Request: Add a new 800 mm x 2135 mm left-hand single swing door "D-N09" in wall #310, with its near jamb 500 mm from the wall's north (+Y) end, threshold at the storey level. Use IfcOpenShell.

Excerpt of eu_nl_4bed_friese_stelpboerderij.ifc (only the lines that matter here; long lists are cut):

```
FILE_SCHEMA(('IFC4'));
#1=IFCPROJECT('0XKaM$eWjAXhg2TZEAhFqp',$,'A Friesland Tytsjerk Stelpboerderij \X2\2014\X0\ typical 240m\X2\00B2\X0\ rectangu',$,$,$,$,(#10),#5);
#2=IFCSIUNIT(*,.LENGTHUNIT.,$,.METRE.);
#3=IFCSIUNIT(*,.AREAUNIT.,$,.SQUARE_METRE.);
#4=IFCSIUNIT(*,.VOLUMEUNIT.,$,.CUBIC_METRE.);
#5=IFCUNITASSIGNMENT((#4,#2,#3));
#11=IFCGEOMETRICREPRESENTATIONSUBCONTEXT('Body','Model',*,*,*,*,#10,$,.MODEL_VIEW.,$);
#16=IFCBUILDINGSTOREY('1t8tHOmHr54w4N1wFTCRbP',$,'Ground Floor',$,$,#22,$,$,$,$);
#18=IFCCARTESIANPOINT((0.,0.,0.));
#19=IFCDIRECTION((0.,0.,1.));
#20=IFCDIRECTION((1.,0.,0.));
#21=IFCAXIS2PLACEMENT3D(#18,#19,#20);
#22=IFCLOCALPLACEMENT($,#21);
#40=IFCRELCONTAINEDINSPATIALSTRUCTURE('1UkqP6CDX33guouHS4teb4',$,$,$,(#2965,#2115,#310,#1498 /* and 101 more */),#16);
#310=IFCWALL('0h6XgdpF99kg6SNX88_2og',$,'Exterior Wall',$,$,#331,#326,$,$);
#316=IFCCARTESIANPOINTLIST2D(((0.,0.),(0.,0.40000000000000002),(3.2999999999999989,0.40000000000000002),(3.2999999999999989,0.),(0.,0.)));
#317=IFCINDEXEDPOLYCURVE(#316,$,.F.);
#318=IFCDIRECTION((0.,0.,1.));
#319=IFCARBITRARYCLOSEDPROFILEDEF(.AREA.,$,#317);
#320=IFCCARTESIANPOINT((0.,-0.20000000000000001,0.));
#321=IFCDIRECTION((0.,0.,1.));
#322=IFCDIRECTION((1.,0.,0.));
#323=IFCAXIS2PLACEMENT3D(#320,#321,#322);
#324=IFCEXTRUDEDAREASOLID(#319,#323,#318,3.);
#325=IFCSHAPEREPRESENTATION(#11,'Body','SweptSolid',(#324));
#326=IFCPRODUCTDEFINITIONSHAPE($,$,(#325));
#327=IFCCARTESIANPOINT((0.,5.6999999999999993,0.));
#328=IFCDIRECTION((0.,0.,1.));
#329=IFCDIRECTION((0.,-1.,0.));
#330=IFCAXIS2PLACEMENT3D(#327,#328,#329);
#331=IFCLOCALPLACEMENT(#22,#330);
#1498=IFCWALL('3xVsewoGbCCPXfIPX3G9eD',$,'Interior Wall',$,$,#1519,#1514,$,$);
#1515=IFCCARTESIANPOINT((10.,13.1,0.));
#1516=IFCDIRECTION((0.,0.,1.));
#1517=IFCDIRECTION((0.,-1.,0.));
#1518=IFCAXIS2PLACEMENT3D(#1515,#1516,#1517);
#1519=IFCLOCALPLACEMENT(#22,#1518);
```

```python
import numpy as np
import ifcopenshell
import ifcopenshell.api.feature
import ifcopenshell.api.geometry
import ifcopenshell.api.root
import ifcopenshell.api.spatial
import ifcopenshell.geom
import ifcopenshell.util.element
import ifcopenshell.util.placement
import ifcopenshell.util.representation
import ifcopenshell.util.shape
import ifcopenshell.util.unit

model = ifcopenshell.open("eu_nl_4bed_friese_stelpboerderij.ifc")
unit_scale = ifcopenshell.util.unit.calculate_unit_scale(model)
settings = ifcopenshell.geom.settings()


def volume(element):
    """Net volume in cubic metres, openings subtracted."""
    shape = ifcopenshell.geom.create_shape(settings, element)
    return ifcopenshell.util.shape.get_volume(shape.geometry)


wall = model.by_guid("0h6XgdpF99kg6SNX88_2og")
storey = ifcopenshell.util.element.get_container(wall, ifc_class="IfcBuildingStorey")
context = ifcopenshell.util.representation.get_context(model, "Model", "Body", "MODEL_VIEW")
before = volume(wall)

width, height, from_end, sill = 0.8, 2.135, 0.5, 0.0  # metres

# The wall runs along its own X axis, and the end named is its -X end.
wall_shape = ifcopenshell.geom.create_shape(settings, wall)
x, y, z = ifcopenshell.util.shape.get_vertices(wall_shape.geometry).T
start = x.min() + from_end
face, thickness = float(y.min()), float(y.max() - y.min())
wall_matrix = ifcopenshell.util.placement.get_local_placement(wall.ObjectPlacement)
level = ifcopenshell.util.placement.get_local_placement(storey.ObjectPlacement)[2, 3]


def in_wall(x, y):
    """Placement at x, y metres in the wall's axes, at sill height."""
    matrix = wall_matrix.copy()
    matrix[:, 3] = wall_matrix @ np.array([x / unit_scale, y / unit_scale, 0.0, 1.0])
    matrix[2, 3] = level + sill / unit_scale
    return matrix


# Opening: a box that overshoots both wall faces by 50 mm.
opening = ifcopenshell.api.root.create_entity(model, ifc_class="IfcOpeningElement", predefined_type="OPENING")
box = ifcopenshell.api.geometry.add_wall_representation(
    model, context=context, length=width, height=height, thickness=thickness + 0.1
)
ifcopenshell.api.geometry.assign_representation(model, product=opening, representation=box)
ifcopenshell.api.geometry.edit_object_placement(model, product=opening, matrix=in_wall(start, face - 0.05), is_si=False)
ifcopenshell.api.feature.add_feature(model, feature=opening, element=wall)

door = ifcopenshell.api.root.create_entity(model, ifc_class="IfcDoor", name="D-N09", predefined_type="DOOR")
door.OverallWidth, door.OverallHeight = width / unit_scale, height / unit_scale
door.OperationType = "SINGLE_SWING_LEFT"
body = ifcopenshell.api.geometry.add_door_representation(
    model,
    context=context,
    overall_width=door.OverallWidth,
    overall_height=door.OverallHeight,
    operation_type="SINGLE_SWING_LEFT",
    lining_properties={"LiningDepth": thickness / unit_scale, "ThresholdDepth": thickness / unit_scale},
)
ifcopenshell.api.geometry.assign_representation(model, product=door, representation=body)
ifcopenshell.api.spatial.assign_container(model, products=[door], relating_structure=storey)
ifcopenshell.api.feature.add_filling(model, opening=opening, element=door)

# The lining spans the wall, so the door starts at the wall face.
ifcopenshell.api.geometry.edit_object_placement(model, product=door, matrix=in_wall(start, face), is_si=False)

after = volume(wall)

print(f"wall volume {before:.3f} -> {after:.3f} m3")

model.write("eu_nl_4bed_friese_stelpboerderij_rev.ifc")
```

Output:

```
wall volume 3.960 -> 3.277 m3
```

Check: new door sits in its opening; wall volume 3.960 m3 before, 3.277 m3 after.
